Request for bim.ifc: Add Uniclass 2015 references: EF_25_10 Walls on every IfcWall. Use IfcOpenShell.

First a look at what the model holds.

```python
import ifcopenshell

model = ifcopenshell.open("bim.ifc")
print(model.schema)
print("classifications:", [c.Name for c in model.by_type("IfcClassification")])
for ifc_class in ("IfcDoor", "IfcRoof", "IfcStair", "IfcWall", "IfcWindow"):
    print(ifc_class, len(model.by_type(ifc_class)))
```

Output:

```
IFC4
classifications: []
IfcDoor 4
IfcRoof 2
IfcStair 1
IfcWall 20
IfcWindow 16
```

```python
import ifcopenshell
import ifcopenshell.api.classification

model = ifcopenshell.open("bim.ifc")

system = ifcopenshell.api.classification.add_classification(model, classification="Uniclass 2015")

codes = {
    "IfcWall": ("EF_25_10", "Walls"),
}
for ifc_class, (code, name) in codes.items():
    products = model.by_type(ifc_class)
    ifcopenshell.api.classification.add_reference(
        model, products=products, classification=system, identification=code, name=name
    )
    print(code, len(products))

model.write("bim_updated.ifc")
```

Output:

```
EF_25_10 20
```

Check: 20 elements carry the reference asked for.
